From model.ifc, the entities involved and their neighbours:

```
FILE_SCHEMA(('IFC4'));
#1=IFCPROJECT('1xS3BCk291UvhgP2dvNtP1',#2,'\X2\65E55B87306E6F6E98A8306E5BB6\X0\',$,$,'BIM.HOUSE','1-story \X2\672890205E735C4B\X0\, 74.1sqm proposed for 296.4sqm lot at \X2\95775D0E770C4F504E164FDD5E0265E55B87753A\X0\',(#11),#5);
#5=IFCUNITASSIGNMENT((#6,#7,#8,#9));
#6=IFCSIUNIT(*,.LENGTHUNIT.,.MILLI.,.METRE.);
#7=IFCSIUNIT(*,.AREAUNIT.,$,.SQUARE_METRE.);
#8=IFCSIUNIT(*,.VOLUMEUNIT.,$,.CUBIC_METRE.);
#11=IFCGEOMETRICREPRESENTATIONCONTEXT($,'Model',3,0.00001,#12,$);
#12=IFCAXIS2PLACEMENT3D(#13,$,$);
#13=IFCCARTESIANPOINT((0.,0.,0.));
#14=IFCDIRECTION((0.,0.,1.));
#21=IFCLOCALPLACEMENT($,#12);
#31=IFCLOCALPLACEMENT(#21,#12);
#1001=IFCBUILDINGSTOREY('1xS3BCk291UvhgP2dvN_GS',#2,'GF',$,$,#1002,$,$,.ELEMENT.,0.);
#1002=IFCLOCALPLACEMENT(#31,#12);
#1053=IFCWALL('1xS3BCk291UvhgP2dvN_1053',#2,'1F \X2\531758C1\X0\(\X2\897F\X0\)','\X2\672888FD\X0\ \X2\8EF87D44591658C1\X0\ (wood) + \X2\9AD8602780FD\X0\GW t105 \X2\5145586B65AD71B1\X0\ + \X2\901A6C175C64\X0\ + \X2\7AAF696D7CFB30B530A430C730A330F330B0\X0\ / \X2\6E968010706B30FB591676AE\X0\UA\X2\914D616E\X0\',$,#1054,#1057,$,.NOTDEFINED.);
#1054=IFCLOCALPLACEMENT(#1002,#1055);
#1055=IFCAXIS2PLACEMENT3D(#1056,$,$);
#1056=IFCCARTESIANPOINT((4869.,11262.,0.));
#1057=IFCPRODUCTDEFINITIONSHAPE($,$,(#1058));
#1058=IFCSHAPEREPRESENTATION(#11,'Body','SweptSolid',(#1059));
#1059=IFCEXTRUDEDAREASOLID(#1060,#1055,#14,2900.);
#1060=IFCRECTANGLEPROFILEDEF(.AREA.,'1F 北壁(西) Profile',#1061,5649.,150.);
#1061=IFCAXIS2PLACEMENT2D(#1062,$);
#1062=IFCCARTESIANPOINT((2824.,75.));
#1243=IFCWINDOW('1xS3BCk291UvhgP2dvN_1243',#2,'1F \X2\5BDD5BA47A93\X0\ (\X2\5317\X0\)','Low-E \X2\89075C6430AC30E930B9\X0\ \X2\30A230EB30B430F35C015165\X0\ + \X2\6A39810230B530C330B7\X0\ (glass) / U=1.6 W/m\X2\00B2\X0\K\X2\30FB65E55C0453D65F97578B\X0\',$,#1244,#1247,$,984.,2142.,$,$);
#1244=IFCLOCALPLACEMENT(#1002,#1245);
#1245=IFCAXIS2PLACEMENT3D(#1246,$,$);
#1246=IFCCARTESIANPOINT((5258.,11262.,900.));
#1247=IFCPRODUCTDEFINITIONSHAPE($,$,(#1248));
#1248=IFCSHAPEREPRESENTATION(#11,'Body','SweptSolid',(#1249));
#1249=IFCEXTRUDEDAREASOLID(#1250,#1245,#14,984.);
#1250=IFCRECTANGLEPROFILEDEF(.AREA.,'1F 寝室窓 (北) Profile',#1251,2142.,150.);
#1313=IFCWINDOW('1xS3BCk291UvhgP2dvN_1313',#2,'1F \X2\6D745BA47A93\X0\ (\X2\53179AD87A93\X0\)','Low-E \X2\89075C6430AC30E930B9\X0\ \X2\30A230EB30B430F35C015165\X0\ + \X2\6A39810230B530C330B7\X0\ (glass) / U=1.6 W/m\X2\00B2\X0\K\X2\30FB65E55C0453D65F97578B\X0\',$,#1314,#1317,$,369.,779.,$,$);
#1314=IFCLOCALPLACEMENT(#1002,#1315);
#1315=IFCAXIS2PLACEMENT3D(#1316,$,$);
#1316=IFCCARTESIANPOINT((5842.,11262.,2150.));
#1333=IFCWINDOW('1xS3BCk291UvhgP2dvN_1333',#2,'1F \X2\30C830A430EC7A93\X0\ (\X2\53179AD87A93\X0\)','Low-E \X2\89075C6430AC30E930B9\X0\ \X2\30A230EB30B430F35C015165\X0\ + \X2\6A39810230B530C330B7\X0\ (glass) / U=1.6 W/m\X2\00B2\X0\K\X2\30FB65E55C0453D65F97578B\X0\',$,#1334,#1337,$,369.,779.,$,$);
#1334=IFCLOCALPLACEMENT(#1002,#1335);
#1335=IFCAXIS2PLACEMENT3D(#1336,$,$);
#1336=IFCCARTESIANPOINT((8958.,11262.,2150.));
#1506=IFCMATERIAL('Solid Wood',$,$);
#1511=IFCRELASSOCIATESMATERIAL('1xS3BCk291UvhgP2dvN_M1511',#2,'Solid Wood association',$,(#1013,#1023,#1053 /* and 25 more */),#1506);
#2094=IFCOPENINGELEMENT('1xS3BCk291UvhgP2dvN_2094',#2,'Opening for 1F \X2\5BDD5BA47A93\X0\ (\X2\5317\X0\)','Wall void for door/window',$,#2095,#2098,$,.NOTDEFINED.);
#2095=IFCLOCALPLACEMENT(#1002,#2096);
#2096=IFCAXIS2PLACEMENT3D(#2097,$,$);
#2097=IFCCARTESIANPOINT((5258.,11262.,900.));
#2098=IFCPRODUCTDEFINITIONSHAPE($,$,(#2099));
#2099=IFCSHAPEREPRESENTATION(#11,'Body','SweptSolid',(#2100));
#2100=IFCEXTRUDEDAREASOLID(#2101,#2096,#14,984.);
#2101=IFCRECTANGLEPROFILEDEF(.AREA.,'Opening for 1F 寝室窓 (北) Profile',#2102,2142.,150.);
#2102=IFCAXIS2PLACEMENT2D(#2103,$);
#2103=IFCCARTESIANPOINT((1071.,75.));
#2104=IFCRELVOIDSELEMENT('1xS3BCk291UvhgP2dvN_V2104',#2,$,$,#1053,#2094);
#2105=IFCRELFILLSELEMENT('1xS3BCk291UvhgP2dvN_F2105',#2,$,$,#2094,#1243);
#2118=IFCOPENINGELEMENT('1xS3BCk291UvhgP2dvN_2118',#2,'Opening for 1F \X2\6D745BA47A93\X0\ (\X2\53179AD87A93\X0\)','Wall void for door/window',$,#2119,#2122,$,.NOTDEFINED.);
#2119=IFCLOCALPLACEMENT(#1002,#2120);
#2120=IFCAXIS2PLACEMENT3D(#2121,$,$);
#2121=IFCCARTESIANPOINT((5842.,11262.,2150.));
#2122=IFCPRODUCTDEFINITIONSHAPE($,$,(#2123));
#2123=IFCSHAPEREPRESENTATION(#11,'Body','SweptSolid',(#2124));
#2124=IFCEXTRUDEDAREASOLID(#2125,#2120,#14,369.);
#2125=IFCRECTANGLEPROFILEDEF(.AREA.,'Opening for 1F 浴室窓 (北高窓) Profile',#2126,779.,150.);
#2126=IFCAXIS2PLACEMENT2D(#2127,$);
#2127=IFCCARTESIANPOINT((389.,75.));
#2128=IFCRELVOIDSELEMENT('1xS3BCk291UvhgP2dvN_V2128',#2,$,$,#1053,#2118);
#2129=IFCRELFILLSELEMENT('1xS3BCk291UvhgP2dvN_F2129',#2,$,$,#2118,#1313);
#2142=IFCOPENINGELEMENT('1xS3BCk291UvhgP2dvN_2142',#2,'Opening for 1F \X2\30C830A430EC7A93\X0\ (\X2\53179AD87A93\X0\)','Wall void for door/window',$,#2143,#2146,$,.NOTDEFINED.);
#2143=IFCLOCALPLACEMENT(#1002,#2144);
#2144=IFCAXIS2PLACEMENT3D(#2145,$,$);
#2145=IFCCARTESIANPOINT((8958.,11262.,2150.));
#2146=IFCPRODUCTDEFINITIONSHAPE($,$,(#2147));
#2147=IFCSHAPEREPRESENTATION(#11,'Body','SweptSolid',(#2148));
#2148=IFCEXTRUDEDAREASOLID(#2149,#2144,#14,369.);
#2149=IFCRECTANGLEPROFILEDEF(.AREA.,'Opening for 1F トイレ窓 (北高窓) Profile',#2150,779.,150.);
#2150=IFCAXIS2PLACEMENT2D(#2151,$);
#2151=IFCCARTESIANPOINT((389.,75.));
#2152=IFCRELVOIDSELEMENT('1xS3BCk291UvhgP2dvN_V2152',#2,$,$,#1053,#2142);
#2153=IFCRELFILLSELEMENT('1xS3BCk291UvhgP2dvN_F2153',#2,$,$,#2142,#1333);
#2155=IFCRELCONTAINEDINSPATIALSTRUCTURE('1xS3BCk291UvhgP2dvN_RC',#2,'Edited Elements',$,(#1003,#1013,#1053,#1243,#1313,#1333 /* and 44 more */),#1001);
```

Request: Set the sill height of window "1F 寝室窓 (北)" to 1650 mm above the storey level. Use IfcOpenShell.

```python
import numpy as np
import ifcopenshell
import ifcopenshell.api.geometry
import ifcopenshell.geom
import ifcopenshell.util.element
import ifcopenshell.util.placement
import ifcopenshell.util.shape
import ifcopenshell.util.unit

model = ifcopenshell.open("model.ifc")
unit_scale = ifcopenshell.util.unit.calculate_unit_scale(model)

window = model.by_id(1243)
opening = window.FillsVoids[0].RelatingOpeningElement
storey = ifcopenshell.util.element.get_container(window, ifc_class="IfcBuildingStorey")
level = ifcopenshell.util.placement.get_local_placement(storey.ObjectPlacement)[2, 3]

# The opening's origin need not be at the sill, so measure its lowest point.
shape = ifcopenshell.geom.create_shape(ifcopenshell.geom.settings(), opening)
bottom = ifcopenshell.util.shape.get_shape_bottom_elevation(shape, shape.geometry) / unit_scale
dz = level + 1.65 / unit_scale - bottom

shift = np.array([0.0, 0.0, dz])
# The window is not placed relative to its opening, so move both.
for product in (opening, window):
    matrix = ifcopenshell.util.placement.get_local_placement(product.ObjectPlacement)
    matrix[:3, 3] += shift
    ifcopenshell.api.geometry.edit_object_placement(model, product=product, matrix=matrix, is_si=False)

print(f"moved by {dz * unit_scale:+.3f} m")

model.write("model_v2.ifc")
```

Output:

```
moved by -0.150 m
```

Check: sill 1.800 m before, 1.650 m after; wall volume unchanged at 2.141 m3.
